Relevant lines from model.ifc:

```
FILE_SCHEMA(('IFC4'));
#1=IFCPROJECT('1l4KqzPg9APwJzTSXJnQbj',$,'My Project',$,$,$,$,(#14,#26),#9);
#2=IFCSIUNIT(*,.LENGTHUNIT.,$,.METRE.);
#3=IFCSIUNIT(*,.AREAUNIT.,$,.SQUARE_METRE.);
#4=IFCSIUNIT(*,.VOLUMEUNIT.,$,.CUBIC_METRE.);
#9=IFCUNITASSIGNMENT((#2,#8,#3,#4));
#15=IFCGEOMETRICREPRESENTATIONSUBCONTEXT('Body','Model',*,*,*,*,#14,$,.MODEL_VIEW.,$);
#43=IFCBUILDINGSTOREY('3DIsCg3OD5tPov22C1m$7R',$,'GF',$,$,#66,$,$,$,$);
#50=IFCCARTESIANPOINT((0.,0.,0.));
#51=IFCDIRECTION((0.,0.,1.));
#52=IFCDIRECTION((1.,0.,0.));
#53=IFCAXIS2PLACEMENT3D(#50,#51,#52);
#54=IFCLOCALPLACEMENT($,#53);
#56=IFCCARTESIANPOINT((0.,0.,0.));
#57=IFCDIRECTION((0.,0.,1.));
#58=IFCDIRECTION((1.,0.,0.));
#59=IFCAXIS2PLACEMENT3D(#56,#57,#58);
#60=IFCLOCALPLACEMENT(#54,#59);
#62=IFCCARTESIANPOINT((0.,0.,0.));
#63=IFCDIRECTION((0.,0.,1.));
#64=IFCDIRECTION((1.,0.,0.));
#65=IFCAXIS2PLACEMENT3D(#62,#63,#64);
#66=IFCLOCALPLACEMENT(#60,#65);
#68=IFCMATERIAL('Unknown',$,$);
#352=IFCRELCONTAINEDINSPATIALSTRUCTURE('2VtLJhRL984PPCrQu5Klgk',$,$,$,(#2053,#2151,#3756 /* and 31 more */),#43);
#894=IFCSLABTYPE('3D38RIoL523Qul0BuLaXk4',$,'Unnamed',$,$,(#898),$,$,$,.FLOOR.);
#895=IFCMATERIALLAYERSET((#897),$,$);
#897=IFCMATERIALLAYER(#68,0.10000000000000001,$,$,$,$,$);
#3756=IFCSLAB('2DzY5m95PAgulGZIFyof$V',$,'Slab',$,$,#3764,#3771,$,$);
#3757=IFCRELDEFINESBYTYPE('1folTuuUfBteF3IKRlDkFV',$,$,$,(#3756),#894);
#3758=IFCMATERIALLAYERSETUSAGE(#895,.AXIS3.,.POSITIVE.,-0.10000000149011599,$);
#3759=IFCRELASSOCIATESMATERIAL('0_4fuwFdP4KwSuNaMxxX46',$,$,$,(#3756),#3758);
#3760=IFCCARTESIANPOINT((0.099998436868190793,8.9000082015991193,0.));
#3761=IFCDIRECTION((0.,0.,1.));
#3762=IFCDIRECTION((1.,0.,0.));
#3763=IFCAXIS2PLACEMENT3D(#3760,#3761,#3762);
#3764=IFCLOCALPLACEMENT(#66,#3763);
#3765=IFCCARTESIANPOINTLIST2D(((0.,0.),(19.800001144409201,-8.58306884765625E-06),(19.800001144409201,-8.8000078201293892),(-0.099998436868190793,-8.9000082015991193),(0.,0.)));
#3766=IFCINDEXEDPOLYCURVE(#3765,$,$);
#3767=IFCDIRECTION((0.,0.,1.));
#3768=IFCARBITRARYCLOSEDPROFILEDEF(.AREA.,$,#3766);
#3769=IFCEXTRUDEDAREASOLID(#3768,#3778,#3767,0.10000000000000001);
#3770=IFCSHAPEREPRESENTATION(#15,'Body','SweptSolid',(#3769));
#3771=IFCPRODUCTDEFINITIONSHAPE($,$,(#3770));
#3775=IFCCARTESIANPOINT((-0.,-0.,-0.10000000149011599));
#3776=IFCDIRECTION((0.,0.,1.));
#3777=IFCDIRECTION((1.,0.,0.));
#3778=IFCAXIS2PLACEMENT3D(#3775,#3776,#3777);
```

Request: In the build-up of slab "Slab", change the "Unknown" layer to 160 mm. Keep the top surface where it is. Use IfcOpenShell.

```python
import ifcopenshell
import ifcopenshell.util.element
import ifcopenshell.util.representation
import ifcopenshell.util.unit

model = ifcopenshell.open("model.ifc")
unit_scale = ifcopenshell.util.unit.calculate_unit_scale(model)

layer_set = model.by_id(895)
layer = next(l for l in layer_set.MaterialLayers if l.Material and l.Material.Name == "Unknown")
change = 0.16 / unit_scale - layer.LayerThickness
layer.LayerThickness += change

# Geometry does not follow the layer set by itself.
slabs = [e for e in ifcopenshell.util.element.get_elements_by_material(model, layer_set) if e.is_a("IfcSlab")]
for slab in sorted(slabs, key=lambda e: e.id()):
    body = ifcopenshell.util.representation.get_representation(slab, "Model", "Body")
    solid = body.Items[0]
    old_depth = solid.Depth
    solid.Depth += change
    # Extruded upwards: lower the start of the extrusion so the top stays.
    x, y, z = solid.Position.Location.Coordinates
    solid.Position.Location = model.createIfcCartesianPoint((x, y, z - change))
    print(slab.id(), f"{old_depth:g} -> {solid.Depth:g}")

# The layers are counted up from the underside, which has moved.
for usage in {ifcopenshell.util.element.get_material(slab) for slab in slabs}:
    usage.OffsetFromReferenceLine -= change

model.write("model_updated.ifc")
```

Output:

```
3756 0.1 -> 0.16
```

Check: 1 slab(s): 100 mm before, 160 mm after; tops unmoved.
